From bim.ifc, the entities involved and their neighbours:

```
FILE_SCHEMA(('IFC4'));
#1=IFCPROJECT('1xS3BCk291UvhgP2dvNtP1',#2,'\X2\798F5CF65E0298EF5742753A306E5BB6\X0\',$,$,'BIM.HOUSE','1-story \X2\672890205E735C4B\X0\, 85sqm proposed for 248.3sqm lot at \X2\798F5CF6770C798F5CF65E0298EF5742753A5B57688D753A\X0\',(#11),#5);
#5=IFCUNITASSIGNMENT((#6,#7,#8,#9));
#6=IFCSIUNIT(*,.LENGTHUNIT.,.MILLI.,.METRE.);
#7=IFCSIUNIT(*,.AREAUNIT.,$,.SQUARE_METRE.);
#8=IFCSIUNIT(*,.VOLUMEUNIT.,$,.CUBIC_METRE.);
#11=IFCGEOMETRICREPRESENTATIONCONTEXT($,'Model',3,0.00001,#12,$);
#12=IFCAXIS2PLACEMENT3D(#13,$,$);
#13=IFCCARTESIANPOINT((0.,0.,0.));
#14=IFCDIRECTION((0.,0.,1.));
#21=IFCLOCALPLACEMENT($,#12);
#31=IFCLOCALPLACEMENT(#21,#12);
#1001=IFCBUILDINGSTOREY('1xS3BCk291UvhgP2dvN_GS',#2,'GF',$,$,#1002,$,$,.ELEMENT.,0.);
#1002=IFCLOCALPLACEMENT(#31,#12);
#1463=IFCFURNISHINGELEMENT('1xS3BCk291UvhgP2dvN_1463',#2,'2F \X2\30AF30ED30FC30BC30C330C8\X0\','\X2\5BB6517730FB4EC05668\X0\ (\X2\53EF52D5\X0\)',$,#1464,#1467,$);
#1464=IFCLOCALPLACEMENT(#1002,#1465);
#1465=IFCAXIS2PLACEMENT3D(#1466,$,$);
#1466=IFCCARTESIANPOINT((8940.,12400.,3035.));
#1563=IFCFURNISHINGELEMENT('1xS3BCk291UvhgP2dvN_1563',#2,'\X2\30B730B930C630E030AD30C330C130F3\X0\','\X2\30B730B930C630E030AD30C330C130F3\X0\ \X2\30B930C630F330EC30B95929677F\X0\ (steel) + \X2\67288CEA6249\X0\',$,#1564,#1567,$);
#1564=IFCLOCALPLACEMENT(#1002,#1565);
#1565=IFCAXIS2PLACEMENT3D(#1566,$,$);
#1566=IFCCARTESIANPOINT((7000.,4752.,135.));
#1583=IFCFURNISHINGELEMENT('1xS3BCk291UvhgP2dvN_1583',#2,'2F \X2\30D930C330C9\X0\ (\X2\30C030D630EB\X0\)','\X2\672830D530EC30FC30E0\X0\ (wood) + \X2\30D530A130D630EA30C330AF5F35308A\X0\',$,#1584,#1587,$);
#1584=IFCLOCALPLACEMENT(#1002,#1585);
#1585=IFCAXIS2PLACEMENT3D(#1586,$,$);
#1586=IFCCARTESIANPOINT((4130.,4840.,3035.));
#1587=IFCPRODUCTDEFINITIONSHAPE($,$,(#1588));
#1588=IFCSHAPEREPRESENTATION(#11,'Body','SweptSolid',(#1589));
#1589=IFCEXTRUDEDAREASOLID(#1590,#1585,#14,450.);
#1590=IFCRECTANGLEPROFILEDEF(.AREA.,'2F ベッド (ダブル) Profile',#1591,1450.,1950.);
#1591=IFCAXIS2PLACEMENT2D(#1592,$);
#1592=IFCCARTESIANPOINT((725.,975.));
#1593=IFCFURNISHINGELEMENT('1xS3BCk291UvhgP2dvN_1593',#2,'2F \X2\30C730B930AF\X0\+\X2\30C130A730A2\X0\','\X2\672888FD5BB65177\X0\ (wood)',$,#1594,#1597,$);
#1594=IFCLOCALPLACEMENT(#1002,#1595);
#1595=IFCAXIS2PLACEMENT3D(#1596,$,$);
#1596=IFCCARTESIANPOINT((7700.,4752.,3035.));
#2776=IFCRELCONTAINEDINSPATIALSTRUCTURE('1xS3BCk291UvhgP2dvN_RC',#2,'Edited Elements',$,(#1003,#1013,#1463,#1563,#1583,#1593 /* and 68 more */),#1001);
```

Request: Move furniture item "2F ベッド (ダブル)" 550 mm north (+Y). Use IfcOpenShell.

```python
import ifcopenshell
import ifcopenshell.api.geometry
import ifcopenshell.util.placement

model = ifcopenshell.open("bim.ifc")

item = model.by_guid("1xS3BCk291UvhgP2dvN_1583")
matrix = ifcopenshell.util.placement.get_local_placement(item.ObjectPlacement)
matrix[1, 3] += 550.0
ifcopenshell.api.geometry.edit_object_placement(model, product=item, matrix=matrix, is_si=False)

print(ifcopenshell.util.placement.get_local_placement(item.ObjectPlacement).round(3) + 0.0)

model.write("bim_v2.ifc")
```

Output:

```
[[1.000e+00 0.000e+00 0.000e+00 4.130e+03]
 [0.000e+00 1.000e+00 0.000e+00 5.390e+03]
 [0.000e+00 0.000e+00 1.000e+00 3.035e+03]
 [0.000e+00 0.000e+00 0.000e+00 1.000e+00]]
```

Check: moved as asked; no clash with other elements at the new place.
